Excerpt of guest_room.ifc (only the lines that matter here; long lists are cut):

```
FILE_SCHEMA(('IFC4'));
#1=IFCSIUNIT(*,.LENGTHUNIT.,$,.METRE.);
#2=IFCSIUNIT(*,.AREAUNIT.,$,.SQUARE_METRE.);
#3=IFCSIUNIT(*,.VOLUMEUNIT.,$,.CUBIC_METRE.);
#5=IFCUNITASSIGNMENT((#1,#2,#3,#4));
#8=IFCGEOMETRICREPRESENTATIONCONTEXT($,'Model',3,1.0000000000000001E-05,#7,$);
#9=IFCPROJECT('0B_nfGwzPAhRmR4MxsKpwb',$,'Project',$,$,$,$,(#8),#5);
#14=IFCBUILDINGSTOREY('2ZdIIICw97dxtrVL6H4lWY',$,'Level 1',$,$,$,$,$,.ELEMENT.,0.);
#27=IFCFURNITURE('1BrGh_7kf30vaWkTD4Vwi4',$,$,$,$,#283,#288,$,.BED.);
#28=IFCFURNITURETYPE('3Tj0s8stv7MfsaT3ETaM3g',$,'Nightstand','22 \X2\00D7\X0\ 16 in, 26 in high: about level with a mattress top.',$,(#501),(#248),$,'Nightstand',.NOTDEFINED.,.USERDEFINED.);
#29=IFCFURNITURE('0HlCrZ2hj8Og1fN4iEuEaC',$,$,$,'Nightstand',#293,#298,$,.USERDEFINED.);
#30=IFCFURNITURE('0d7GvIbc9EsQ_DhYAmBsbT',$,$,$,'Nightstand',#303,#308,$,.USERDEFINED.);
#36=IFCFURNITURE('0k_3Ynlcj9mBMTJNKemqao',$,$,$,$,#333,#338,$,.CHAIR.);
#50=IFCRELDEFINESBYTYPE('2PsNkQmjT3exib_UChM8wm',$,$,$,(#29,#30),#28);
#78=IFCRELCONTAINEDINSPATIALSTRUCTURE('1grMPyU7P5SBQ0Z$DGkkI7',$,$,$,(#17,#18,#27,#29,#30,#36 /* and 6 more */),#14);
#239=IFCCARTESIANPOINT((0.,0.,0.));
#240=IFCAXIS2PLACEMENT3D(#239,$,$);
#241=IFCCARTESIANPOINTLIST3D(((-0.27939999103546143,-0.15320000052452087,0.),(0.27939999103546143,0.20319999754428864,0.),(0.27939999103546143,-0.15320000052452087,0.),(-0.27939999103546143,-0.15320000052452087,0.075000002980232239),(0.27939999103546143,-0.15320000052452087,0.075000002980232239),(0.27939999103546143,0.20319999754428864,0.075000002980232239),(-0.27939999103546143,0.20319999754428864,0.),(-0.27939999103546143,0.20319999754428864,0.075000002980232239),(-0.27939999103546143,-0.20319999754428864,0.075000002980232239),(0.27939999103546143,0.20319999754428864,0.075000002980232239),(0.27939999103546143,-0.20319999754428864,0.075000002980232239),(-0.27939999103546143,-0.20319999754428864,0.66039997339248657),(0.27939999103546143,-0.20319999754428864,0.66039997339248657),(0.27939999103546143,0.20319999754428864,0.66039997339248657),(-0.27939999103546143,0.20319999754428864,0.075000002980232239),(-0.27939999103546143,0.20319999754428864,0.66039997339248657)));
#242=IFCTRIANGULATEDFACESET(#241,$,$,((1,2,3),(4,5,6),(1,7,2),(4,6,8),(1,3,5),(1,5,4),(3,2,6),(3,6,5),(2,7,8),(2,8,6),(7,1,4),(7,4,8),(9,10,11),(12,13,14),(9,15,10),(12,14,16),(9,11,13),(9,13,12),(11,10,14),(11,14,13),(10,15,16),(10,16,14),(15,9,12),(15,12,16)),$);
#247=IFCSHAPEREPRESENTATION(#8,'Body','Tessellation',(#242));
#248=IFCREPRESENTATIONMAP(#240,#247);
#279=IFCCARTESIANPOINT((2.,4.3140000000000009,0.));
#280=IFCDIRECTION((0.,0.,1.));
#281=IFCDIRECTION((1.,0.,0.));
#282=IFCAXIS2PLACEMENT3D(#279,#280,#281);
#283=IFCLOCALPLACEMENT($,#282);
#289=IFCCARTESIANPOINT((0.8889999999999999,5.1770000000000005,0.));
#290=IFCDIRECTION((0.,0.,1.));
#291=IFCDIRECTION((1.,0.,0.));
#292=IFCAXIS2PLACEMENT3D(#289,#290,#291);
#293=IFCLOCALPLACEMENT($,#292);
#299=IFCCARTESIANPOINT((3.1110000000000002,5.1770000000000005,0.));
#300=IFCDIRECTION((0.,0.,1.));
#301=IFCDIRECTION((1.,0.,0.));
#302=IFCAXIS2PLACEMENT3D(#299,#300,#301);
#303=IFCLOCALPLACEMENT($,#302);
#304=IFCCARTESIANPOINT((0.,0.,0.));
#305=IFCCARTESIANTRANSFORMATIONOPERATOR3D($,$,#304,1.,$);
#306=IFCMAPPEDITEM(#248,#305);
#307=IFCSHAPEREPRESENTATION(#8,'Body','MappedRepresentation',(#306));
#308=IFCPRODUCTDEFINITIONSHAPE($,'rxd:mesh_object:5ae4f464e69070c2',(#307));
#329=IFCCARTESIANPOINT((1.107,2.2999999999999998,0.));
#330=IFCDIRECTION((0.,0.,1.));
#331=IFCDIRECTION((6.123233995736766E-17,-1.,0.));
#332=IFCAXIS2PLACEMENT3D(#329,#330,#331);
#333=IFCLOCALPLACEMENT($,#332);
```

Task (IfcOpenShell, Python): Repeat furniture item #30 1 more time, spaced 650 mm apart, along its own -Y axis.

```python
import ifcopenshell
import ifcopenshell.api.geometry
import ifcopenshell.api.root
import ifcopenshell.util.element
import ifcopenshell.util.placement

model = ifcopenshell.open("guest_room.ifc")

source = model.by_guid("0d7GvIbc9EsQ_DhYAmBsbT")
base = ifcopenshell.util.placement.get_local_placement(source.ObjectPlacement)
step = -base[:3, 1] * 0.65

for i in range(1, 2):
    copy = ifcopenshell.api.root.copy_class(model, product=source)
    copy.Representation = ifcopenshell.util.element.copy_deep(
        model, source.Representation, exclude=["IfcGeometricRepresentationContext", "IfcRepresentationMap"]
    )
    matrix = base.copy()
    matrix[:3, 3] += i * step
    print("added at", matrix[:3, 3].round(3) + 0.0)
    ifcopenshell.api.geometry.edit_object_placement(model, product=copy, matrix=matrix, is_si=False)

model.write("guest_room_v2.ifc")
```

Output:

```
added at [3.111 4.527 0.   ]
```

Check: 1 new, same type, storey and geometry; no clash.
